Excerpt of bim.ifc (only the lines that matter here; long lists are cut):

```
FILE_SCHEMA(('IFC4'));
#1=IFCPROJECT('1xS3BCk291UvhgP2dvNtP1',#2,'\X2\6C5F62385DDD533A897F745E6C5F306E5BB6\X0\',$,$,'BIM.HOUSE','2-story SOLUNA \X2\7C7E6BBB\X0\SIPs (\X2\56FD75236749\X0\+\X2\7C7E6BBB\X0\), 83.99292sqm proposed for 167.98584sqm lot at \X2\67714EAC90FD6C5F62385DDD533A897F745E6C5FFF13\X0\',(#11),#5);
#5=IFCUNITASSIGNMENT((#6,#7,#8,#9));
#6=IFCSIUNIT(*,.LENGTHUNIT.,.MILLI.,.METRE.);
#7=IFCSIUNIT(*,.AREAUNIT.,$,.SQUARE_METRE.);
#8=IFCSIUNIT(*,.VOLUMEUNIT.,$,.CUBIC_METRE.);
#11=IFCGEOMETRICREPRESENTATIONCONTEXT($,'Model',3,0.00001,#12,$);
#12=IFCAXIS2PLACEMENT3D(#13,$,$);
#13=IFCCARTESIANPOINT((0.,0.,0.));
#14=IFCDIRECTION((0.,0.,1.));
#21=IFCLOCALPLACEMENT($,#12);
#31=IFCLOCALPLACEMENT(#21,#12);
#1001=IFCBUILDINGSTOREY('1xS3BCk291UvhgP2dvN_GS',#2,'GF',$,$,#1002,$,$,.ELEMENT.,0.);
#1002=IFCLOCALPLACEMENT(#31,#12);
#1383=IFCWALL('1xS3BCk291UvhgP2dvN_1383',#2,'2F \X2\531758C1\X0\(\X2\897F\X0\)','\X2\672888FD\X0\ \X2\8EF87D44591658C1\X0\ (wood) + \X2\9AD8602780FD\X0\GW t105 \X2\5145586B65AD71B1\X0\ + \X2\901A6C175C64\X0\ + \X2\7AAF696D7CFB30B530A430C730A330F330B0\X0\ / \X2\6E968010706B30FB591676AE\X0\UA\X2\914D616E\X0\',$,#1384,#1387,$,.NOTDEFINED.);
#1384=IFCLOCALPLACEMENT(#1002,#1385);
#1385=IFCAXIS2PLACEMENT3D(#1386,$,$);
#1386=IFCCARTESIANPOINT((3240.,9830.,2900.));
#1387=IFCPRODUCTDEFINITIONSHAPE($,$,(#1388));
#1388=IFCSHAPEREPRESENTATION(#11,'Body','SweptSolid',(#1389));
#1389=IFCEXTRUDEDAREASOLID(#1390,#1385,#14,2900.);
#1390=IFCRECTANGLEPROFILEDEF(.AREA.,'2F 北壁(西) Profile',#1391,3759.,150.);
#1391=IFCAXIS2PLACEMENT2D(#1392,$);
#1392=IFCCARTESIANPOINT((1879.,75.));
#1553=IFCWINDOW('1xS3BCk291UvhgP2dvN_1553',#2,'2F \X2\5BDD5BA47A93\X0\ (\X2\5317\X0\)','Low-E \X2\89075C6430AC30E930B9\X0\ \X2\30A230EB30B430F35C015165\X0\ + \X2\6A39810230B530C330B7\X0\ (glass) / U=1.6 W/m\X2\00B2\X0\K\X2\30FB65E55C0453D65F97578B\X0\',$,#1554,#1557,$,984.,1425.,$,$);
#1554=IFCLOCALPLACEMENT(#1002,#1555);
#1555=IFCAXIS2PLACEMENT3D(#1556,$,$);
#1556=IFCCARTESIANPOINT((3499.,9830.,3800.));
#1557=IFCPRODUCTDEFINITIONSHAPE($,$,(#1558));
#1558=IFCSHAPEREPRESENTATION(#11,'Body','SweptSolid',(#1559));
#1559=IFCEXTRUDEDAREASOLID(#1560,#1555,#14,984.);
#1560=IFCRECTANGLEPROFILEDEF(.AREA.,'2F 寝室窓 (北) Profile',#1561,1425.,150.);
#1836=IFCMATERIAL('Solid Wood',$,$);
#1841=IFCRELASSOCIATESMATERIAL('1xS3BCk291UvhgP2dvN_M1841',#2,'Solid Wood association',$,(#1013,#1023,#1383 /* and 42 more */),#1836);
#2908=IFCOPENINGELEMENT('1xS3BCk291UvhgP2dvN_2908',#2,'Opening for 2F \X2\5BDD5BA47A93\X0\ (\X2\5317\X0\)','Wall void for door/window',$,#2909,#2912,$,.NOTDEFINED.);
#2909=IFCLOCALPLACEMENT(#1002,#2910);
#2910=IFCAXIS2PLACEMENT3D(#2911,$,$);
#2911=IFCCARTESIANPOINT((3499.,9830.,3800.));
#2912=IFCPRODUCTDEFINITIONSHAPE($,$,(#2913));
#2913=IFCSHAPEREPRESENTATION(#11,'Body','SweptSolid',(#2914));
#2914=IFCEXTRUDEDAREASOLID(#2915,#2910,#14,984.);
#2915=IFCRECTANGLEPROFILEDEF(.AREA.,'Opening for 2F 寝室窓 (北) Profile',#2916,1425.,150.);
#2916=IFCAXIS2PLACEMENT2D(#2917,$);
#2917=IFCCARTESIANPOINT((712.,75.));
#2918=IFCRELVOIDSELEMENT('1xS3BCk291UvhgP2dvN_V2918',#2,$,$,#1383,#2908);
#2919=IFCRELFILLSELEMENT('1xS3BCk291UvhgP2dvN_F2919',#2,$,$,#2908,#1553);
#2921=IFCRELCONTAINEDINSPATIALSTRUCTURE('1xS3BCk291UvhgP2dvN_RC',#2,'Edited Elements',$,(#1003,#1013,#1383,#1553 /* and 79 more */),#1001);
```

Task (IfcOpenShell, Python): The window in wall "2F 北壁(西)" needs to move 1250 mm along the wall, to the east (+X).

```python
import ifcopenshell
import ifcopenshell.api.geometry
import ifcopenshell.util.placement
import ifcopenshell.util.unit

model = ifcopenshell.open("bim.ifc")
unit_scale = ifcopenshell.util.unit.calculate_unit_scale(model)

window = model.by_guid("1xS3BCk291UvhgP2dvN_1553")
opening = window.FillsVoids[0].RelatingOpeningElement
wall = opening.VoidsElements[0].RelatingBuildingElement

wall_matrix = ifcopenshell.util.placement.get_local_placement(wall.ObjectPlacement)
shift = wall_matrix[:3, 0] * 1.25 / unit_scale
before = ifcopenshell.util.placement.get_local_placement(window.ObjectPlacement)[:3, 3].copy()

# The window is not placed relative to its opening, so move both.
for product in (opening, window):
    matrix = ifcopenshell.util.placement.get_local_placement(product.ObjectPlacement)
    matrix[:3, 3] += shift
    ifcopenshell.api.geometry.edit_object_placement(model, product=product, matrix=matrix, is_si=False)

after = ifcopenshell.util.placement.get_local_placement(window.ObjectPlacement)[:3, 3]
print("window moved by", (after - before).round(3) + 0.0)

model.write("bim_edited.ifc")
```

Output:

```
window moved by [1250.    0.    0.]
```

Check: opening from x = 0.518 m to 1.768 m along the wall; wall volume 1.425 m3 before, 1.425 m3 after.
